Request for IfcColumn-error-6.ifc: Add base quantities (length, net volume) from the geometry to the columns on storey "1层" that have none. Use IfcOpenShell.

First a look at what the model holds.

```python
import ifcopenshell
import ifcopenshell.util.element
import ifcopenshell.util.unit

model = ifcopenshell.open("IfcColumn-error-6.ifc")
print(model.schema)
for unit_type in ("LENGTHUNIT", "AREAUNIT", "VOLUMEUNIT"):
    print(unit_type, ifcopenshell.util.unit.calculate_unit_scale(model, unit_type))
storey = next(s for s in model.by_type("IfcBuildingStorey") if s.Name == "1层")
columns = [e for e in ifcopenshell.util.element.get_decomposition(storey) if e.is_a("IfcColumn")]
for e in sorted(columns, key=lambda e: e.id()):
    print(e.id(), e.is_a(), e.Name, list(ifcopenshell.util.element.get_psets(e, qtos_only=True)), sep=" | ")
```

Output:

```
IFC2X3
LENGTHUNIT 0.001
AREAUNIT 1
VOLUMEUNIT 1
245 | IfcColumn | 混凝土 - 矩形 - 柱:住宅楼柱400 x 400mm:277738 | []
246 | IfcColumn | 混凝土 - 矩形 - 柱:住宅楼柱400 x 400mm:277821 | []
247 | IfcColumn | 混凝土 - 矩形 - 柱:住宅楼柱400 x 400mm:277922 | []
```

```python
import ifcopenshell
import ifcopenshell.api.pset
import ifcopenshell.geom
import ifcopenshell.util.element
import ifcopenshell.util.shape
import ifcopenshell.util.unit

model = ifcopenshell.open("IfcColumn-error-6.ifc")
unit_scale = ifcopenshell.util.unit.calculate_unit_scale(model)
volume_scale = ifcopenshell.util.unit.calculate_unit_scale(model, "VOLUMEUNIT")
settings = ifcopenshell.geom.settings()

storey = next(s for s in model.by_type("IfcBuildingStorey") if s.Name == "1层")
columns = [e for e in ifcopenshell.util.element.get_decomposition(storey) if e.is_a("IfcColumn")]

for e in sorted(columns, key=lambda e: e.id()):
    if ifcopenshell.util.element.get_psets(e, qtos_only=True, should_inherit=False):
        continue
    # Geometry comes back in metres, in the element's own axes.
    shape = ifcopenshell.geom.create_shape(settings, e)
    values = {
        "Length": ifcopenshell.util.shape.get_z(shape.geometry) / unit_scale,
        "NetVolume": ifcopenshell.util.shape.get_volume(shape.geometry) / volume_scale,
    }
    qto = ifcopenshell.api.pset.add_qto(model, product=e, name="BaseQuantities")
    ifcopenshell.api.pset.edit_qto(model, qto=qto, properties=values)
    print(e.id(), {k: round(v, 3) for k, v in values.items()})

model.write("IfcColumn-error-6_rev.ifc")
```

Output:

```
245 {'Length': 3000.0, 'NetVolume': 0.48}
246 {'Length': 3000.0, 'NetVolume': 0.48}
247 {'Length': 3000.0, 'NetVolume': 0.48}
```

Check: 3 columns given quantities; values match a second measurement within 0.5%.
